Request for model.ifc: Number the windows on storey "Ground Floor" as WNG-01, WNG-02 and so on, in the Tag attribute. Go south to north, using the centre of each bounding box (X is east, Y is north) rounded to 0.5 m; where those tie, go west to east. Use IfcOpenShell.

First a look at what the model holds.

```python
import ifcopenshell
import ifcopenshell.util.element
import ifcopenshell.util.placement

model = ifcopenshell.open("model.ifc")
print(model.schema)
storey = next(s for s in model.by_type("IfcBuildingStorey") if s.Name == "Ground Floor")
windows = [e for e in ifcopenshell.util.element.get_decomposition(storey) if e.is_a("IfcWindow")]
for e in sorted(windows, key=lambda e: e.id()):
    origin = ifcopenshell.util.placement.get_local_placement(e.ObjectPlacement)[:3, 3]
    print(e.id(), e.Tag, e.Name, origin.round(2) + 0.0, sep=" | ")
```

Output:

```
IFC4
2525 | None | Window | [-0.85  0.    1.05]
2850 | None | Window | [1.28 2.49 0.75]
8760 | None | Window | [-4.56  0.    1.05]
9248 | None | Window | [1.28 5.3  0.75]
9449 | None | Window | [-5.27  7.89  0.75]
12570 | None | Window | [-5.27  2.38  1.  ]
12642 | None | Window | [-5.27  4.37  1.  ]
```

```python
import ifcopenshell
import ifcopenshell.geom
import ifcopenshell.util.element
import ifcopenshell.util.shape

model = ifcopenshell.open("model.ifc")
settings = ifcopenshell.geom.settings()
settings.set("use-world-coords", True)


def centre(element):
    shape = ifcopenshell.geom.create_shape(settings, element)
    return ifcopenshell.util.shape.get_bbox_centroid(shape.geometry)


storey = next(s for s in model.by_type("IfcBuildingStorey") if s.Name == "Ground Floor")
windows = [e for e in ifcopenshell.util.element.get_decomposition(storey) if e.is_a("IfcWindow")]

# Insertion points can sit at a corner or the storey origin, so sort by the geometry (in metres).
centres = {e: centre(e) for e in windows}
windows.sort(key=lambda e: (round(centres[e][1] / 0.5), centres[e][0]))

for i, e in enumerate(windows, start=1):
    number = f"WNG-{i:02d}"
    e.Tag = number
    print(e.id(), number)

model.write("model_rev.ifc")
```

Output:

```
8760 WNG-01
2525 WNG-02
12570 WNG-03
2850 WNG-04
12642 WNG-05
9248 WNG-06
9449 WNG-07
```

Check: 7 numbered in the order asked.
